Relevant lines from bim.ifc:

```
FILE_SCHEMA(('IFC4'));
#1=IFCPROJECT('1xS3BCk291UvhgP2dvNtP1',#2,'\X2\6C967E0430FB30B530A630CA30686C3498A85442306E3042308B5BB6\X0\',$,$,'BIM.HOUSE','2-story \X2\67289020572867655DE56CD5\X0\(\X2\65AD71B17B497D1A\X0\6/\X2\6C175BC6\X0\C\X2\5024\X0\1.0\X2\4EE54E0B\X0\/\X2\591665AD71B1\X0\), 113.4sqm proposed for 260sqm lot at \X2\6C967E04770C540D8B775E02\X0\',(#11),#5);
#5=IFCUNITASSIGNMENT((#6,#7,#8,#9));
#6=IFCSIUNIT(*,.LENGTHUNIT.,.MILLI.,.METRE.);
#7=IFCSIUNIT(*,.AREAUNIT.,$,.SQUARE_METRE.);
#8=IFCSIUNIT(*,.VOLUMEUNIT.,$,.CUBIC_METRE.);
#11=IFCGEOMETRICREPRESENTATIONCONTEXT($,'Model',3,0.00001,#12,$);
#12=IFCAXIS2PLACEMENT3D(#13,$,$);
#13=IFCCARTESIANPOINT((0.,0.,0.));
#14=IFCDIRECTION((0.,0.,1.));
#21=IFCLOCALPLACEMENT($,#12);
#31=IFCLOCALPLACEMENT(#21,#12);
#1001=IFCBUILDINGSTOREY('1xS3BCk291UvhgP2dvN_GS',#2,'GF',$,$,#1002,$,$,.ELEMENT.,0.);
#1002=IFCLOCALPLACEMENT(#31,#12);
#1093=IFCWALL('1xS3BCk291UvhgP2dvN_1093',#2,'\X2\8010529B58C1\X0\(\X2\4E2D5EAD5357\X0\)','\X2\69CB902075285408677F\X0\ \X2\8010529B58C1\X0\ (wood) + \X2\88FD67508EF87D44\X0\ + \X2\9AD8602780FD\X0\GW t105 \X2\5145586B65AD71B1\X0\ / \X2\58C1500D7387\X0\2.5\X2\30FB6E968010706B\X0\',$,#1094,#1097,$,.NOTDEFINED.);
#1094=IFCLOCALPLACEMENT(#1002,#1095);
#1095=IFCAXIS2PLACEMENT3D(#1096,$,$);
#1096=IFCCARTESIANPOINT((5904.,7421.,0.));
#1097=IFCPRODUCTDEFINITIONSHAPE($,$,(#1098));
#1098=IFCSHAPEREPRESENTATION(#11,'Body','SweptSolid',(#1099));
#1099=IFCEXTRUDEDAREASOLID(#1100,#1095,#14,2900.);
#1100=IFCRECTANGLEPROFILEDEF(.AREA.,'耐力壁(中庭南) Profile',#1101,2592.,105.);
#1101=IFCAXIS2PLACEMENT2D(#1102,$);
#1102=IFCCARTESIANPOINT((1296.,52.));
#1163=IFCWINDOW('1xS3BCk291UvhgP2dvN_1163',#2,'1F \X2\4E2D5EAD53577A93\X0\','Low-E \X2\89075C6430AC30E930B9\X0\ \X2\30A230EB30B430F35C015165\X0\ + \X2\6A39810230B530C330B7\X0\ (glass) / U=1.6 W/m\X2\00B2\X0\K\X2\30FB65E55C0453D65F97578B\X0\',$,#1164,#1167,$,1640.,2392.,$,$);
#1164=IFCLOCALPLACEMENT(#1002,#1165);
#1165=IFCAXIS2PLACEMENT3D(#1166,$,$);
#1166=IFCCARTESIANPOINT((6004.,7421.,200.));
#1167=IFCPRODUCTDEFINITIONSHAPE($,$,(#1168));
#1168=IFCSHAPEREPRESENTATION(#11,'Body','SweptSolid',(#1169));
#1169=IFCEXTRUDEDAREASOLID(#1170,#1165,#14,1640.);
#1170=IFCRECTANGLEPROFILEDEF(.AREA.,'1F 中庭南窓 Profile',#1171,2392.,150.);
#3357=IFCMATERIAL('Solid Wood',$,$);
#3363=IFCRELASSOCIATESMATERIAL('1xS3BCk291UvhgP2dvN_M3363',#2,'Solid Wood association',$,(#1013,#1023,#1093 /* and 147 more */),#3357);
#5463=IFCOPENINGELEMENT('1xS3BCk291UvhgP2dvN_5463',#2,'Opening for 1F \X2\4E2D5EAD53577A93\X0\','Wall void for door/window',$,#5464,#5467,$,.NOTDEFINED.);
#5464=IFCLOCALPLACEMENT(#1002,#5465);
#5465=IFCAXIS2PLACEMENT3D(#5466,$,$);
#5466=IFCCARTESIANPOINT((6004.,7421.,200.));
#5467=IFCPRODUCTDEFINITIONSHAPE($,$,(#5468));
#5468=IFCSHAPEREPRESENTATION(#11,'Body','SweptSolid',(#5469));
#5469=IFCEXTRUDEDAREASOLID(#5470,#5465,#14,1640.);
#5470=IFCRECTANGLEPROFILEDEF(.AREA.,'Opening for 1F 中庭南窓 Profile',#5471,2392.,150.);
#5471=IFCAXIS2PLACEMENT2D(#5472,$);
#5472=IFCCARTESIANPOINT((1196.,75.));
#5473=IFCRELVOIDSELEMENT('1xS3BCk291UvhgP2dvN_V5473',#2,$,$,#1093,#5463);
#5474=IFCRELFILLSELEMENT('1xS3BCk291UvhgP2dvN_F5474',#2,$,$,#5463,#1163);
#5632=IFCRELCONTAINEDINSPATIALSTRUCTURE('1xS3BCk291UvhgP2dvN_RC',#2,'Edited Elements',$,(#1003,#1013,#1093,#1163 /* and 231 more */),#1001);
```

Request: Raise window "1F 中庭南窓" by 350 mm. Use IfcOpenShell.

```python
import numpy as np
import ifcopenshell
import ifcopenshell.api.geometry
import ifcopenshell.util.placement
import ifcopenshell.util.unit

model = ifcopenshell.open("bim.ifc")
unit_scale = ifcopenshell.util.unit.calculate_unit_scale(model)

window = model.by_id(1163)
opening = window.FillsVoids[0].RelatingOpeningElement
dz = 0.35 / unit_scale

shift = np.array([0.0, 0.0, dz])
# The window is not placed relative to its opening, so move both.
for product in (opening, window):
    matrix = ifcopenshell.util.placement.get_local_placement(product.ObjectPlacement)
    matrix[:3, 3] += shift
    ifcopenshell.api.geometry.edit_object_placement(model, product=product, matrix=matrix, is_si=False)

print(f"moved by {dz * unit_scale:+.3f} m")

model.write("bim_rev.ifc")
```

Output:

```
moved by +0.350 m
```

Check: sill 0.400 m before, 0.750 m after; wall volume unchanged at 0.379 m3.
